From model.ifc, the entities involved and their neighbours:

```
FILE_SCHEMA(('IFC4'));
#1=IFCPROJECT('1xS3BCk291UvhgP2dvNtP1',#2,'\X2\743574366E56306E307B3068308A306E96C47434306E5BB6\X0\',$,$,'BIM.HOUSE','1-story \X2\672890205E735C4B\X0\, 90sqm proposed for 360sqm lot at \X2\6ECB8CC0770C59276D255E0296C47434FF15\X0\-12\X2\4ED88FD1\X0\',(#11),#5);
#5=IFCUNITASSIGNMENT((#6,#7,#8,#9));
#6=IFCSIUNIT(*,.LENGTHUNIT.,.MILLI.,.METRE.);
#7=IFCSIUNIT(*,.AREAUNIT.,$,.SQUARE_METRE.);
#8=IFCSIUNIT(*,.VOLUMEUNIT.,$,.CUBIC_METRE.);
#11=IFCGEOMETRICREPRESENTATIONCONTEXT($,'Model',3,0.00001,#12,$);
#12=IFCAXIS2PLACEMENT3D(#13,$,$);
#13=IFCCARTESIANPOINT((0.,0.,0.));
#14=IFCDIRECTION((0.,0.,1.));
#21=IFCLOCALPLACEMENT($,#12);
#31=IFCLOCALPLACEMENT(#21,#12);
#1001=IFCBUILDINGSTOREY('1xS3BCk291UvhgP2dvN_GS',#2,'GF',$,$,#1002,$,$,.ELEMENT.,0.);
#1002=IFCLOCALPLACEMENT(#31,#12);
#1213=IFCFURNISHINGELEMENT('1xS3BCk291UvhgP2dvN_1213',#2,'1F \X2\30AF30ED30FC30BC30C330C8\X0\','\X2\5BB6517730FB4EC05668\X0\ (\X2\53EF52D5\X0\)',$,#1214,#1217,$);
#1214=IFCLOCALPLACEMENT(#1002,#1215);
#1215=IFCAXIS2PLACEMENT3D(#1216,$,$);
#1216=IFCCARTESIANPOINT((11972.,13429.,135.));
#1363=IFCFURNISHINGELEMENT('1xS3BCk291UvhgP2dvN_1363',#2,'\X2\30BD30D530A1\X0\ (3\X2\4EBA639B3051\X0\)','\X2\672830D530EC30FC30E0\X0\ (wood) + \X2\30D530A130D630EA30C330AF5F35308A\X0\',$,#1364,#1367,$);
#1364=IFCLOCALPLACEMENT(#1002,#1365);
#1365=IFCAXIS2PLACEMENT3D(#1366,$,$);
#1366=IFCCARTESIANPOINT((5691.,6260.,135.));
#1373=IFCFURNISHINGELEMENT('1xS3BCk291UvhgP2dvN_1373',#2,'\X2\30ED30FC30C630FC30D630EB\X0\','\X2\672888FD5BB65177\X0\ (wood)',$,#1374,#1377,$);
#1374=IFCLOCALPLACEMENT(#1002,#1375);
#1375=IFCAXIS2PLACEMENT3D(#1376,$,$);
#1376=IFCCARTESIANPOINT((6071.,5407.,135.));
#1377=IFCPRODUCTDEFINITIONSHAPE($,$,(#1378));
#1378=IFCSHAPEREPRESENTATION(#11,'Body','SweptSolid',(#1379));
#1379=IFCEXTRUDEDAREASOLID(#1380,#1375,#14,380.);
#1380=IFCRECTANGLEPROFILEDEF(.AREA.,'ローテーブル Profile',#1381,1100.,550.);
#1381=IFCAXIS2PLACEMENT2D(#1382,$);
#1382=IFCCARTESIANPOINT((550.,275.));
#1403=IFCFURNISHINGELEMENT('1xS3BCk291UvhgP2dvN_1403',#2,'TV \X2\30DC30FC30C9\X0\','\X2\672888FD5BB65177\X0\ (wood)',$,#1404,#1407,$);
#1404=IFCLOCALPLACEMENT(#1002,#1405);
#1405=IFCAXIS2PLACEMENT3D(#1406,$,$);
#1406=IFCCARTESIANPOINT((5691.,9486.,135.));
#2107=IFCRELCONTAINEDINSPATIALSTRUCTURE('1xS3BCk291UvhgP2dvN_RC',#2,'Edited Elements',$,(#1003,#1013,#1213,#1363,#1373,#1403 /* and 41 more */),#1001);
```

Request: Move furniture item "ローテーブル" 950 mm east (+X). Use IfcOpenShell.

```python
import ifcopenshell
import ifcopenshell.api.geometry
import ifcopenshell.util.placement
import ifcopenshell.util.unit

model = ifcopenshell.open("model.ifc")
unit_scale = ifcopenshell.util.unit.calculate_unit_scale(model)

item = model.by_guid("1xS3BCk291UvhgP2dvN_1373")
matrix = ifcopenshell.util.placement.get_local_placement(item.ObjectPlacement)
matrix[0, 3] += 0.95 / unit_scale
ifcopenshell.api.geometry.edit_object_placement(model, product=item, matrix=matrix, is_si=False)

print(ifcopenshell.util.placement.get_local_placement(item.ObjectPlacement).round(3) + 0.0)

model.write("model_updated.ifc")
```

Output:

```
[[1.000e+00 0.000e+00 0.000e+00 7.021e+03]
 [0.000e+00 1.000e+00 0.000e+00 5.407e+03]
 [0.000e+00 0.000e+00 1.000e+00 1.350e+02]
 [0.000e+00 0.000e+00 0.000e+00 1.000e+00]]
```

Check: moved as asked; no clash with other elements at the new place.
